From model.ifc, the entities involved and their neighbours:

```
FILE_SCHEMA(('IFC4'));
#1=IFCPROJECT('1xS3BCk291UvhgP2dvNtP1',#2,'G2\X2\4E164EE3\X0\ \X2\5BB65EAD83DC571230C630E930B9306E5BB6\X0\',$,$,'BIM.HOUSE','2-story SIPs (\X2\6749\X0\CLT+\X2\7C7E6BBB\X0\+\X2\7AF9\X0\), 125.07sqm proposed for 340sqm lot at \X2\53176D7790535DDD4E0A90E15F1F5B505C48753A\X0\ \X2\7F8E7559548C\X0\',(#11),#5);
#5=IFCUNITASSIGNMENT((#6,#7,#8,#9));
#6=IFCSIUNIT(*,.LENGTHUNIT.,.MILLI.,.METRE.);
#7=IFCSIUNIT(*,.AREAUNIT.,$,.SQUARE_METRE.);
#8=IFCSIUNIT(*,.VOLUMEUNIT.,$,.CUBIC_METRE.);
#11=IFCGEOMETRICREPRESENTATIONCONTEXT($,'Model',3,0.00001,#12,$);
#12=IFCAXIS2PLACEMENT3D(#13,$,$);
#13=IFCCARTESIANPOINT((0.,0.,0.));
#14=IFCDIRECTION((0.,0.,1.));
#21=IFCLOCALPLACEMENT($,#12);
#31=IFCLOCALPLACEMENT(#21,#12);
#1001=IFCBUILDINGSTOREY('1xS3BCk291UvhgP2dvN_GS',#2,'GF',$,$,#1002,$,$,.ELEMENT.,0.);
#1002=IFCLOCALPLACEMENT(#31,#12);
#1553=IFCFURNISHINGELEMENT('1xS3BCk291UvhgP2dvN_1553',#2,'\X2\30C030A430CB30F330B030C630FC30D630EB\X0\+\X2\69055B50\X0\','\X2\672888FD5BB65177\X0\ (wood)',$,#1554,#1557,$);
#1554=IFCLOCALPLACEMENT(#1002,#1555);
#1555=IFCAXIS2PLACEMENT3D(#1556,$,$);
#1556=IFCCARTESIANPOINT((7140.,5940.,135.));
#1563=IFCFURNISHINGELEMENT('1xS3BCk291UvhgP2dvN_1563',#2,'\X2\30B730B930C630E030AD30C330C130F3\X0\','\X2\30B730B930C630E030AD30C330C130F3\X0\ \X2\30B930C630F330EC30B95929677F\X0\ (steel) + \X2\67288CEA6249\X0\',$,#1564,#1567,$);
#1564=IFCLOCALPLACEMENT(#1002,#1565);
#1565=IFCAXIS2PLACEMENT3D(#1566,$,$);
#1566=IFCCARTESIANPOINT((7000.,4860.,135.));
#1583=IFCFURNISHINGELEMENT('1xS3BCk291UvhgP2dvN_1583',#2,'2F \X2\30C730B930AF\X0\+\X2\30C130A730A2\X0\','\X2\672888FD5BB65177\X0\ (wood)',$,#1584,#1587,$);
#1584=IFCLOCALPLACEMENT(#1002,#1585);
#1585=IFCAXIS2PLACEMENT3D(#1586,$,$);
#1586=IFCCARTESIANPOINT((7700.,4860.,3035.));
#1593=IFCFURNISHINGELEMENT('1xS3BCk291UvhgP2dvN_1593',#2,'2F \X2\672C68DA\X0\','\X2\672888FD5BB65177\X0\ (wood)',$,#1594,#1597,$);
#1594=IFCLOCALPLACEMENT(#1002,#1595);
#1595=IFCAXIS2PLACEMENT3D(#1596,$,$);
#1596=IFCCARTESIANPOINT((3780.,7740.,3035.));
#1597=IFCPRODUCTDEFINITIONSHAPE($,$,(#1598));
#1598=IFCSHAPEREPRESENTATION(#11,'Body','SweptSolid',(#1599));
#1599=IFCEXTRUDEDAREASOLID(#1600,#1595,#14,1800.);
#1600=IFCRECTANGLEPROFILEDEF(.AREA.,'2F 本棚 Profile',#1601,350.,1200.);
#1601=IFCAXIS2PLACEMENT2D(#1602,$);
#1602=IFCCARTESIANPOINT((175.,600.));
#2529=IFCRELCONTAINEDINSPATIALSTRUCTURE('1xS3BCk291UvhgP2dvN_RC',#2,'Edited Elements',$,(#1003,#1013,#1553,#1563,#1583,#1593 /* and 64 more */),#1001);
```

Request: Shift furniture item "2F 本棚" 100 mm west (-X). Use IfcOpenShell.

```python
import ifcopenshell
import ifcopenshell.api.geometry
import ifcopenshell.util.placement

model = ifcopenshell.open("model.ifc")

item = model.by_guid("1xS3BCk291UvhgP2dvN_1593")
matrix = ifcopenshell.util.placement.get_local_placement(item.ObjectPlacement)
matrix[0, 3] -= 100.0
ifcopenshell.api.geometry.edit_object_placement(model, product=item, matrix=matrix, is_si=False)

print(ifcopenshell.util.placement.get_local_placement(item.ObjectPlacement).round(3) + 0.0)

model.write("model-out.ifc")
```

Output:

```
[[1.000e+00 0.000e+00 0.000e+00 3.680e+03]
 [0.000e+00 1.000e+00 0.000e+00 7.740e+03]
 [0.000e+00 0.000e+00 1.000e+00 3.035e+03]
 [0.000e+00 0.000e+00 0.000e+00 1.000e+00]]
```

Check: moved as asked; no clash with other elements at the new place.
